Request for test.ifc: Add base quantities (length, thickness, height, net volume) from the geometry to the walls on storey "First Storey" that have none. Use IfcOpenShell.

First a look at what the model holds.

```python
import ifcopenshell
import ifcopenshell.util.element
import ifcopenshell.util.unit

model = ifcopenshell.open("test.ifc")
print(model.schema)
for unit_type in ("LENGTHUNIT", "AREAUNIT", "VOLUMEUNIT"):
    print(unit_type, ifcopenshell.util.unit.calculate_unit_scale(model, unit_type))
storey = next(s for s in model.by_type("IfcBuildingStorey") if s.Name == "First Storey")
walls = [e for e in ifcopenshell.util.element.get_decomposition(storey) if e.is_a("IfcWall")]
for e in sorted(walls, key=lambda e: e.id()):
    print(e.id(), e.is_a(), e.Name, list(ifcopenshell.util.element.get_psets(e, qtos_only=True)), sep=" | ")
```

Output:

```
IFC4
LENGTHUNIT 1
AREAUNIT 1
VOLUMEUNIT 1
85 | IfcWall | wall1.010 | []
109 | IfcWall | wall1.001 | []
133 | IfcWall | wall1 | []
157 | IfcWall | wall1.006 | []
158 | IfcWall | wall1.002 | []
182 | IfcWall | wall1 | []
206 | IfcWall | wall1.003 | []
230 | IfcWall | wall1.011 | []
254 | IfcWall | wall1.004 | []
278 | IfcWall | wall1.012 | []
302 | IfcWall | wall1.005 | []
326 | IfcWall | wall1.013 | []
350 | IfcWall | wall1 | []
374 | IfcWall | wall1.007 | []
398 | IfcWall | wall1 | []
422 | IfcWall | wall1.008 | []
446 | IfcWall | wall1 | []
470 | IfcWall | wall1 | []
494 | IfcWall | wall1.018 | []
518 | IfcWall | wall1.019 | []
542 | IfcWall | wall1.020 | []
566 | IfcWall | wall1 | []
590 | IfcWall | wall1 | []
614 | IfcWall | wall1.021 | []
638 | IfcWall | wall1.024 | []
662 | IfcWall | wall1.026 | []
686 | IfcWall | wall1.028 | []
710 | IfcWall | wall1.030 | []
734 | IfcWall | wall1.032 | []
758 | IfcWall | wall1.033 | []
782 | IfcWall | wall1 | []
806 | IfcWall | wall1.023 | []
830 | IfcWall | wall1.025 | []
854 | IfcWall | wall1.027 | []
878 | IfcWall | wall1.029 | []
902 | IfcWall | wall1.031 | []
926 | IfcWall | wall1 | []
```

```python
import ifcopenshell
import ifcopenshell.api.pset
import ifcopenshell.geom
import ifcopenshell.util.element
import ifcopenshell.util.shape
import ifcopenshell.util.unit

model = ifcopenshell.open("test.ifc")
unit_scale = ifcopenshell.util.unit.calculate_unit_scale(model)
volume_scale = ifcopenshell.util.unit.calculate_unit_scale(model, "VOLUMEUNIT")
settings = ifcopenshell.geom.settings()

storey = next(s for s in model.by_type("IfcBuildingStorey") if s.Name == "First Storey")
walls = [e for e in ifcopenshell.util.element.get_decomposition(storey) if e.is_a("IfcWall")]

for e in sorted(walls, key=lambda e: e.id()):
    if ifcopenshell.util.element.get_psets(e, qtos_only=True, should_inherit=False):
        continue
    # Geometry comes back in metres, in the element's own axes.
    shape = ifcopenshell.geom.create_shape(settings, e)
    values = {
        "Length": ifcopenshell.util.shape.get_x(shape.geometry) / unit_scale,
        "Width": ifcopenshell.util.shape.get_y(shape.geometry) / unit_scale,
        "Height": ifcopenshell.util.shape.get_z(shape.geometry) / unit_scale,
        "NetVolume": ifcopenshell.util.shape.get_volume(shape.geometry) / volume_scale,
    }
    qto = ifcopenshell.api.pset.add_qto(model, product=e, name="Qto_WallBaseQuantities")
    ifcopenshell.api.pset.edit_qto(model, qto=qto, properties=values)
    print(e.id(), {k: round(v, 3) for k, v in values.items()})

model.write("test-out.ifc")
```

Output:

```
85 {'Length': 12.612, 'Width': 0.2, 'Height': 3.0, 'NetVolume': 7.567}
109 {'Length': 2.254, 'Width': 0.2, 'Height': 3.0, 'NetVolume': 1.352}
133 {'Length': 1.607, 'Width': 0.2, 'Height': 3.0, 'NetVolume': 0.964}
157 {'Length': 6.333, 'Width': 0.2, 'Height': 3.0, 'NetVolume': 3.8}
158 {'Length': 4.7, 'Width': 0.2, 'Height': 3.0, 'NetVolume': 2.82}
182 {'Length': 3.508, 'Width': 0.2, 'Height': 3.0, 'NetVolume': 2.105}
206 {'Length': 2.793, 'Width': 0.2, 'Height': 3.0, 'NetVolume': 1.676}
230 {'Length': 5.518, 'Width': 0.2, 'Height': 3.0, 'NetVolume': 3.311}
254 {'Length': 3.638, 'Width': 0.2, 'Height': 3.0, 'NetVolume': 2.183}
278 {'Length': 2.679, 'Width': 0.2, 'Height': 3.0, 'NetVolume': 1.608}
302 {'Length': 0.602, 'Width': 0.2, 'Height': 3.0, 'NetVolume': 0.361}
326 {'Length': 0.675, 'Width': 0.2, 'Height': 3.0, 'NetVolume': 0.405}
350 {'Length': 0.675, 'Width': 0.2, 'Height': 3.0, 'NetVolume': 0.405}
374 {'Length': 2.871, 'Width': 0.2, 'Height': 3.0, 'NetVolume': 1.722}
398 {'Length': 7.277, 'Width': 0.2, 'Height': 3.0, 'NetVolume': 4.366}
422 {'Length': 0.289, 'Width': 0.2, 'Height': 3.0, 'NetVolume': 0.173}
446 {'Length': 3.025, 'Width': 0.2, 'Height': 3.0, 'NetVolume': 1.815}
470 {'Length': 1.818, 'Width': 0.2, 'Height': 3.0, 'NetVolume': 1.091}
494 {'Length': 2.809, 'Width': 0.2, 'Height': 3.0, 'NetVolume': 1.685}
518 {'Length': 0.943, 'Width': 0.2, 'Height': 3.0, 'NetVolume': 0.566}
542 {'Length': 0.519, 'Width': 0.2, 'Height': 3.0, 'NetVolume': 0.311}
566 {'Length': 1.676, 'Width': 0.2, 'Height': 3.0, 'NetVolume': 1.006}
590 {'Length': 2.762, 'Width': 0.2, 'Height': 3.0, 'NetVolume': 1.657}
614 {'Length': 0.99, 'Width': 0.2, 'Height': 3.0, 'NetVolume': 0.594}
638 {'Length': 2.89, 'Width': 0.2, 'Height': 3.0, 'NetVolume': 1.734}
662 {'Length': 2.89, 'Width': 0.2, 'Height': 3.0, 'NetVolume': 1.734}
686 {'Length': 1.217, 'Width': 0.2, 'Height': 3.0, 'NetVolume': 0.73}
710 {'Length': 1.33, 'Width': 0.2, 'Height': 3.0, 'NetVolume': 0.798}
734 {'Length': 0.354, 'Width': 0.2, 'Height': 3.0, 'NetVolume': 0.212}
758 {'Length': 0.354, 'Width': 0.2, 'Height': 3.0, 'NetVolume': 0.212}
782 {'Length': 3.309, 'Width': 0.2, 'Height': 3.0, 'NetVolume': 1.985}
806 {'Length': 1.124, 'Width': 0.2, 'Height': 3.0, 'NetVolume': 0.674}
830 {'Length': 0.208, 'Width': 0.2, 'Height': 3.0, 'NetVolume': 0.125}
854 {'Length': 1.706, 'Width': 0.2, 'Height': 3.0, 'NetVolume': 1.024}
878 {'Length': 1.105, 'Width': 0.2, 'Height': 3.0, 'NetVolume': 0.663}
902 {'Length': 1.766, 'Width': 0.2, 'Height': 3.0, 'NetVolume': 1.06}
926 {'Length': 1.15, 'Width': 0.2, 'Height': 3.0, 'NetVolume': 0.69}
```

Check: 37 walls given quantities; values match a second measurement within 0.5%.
